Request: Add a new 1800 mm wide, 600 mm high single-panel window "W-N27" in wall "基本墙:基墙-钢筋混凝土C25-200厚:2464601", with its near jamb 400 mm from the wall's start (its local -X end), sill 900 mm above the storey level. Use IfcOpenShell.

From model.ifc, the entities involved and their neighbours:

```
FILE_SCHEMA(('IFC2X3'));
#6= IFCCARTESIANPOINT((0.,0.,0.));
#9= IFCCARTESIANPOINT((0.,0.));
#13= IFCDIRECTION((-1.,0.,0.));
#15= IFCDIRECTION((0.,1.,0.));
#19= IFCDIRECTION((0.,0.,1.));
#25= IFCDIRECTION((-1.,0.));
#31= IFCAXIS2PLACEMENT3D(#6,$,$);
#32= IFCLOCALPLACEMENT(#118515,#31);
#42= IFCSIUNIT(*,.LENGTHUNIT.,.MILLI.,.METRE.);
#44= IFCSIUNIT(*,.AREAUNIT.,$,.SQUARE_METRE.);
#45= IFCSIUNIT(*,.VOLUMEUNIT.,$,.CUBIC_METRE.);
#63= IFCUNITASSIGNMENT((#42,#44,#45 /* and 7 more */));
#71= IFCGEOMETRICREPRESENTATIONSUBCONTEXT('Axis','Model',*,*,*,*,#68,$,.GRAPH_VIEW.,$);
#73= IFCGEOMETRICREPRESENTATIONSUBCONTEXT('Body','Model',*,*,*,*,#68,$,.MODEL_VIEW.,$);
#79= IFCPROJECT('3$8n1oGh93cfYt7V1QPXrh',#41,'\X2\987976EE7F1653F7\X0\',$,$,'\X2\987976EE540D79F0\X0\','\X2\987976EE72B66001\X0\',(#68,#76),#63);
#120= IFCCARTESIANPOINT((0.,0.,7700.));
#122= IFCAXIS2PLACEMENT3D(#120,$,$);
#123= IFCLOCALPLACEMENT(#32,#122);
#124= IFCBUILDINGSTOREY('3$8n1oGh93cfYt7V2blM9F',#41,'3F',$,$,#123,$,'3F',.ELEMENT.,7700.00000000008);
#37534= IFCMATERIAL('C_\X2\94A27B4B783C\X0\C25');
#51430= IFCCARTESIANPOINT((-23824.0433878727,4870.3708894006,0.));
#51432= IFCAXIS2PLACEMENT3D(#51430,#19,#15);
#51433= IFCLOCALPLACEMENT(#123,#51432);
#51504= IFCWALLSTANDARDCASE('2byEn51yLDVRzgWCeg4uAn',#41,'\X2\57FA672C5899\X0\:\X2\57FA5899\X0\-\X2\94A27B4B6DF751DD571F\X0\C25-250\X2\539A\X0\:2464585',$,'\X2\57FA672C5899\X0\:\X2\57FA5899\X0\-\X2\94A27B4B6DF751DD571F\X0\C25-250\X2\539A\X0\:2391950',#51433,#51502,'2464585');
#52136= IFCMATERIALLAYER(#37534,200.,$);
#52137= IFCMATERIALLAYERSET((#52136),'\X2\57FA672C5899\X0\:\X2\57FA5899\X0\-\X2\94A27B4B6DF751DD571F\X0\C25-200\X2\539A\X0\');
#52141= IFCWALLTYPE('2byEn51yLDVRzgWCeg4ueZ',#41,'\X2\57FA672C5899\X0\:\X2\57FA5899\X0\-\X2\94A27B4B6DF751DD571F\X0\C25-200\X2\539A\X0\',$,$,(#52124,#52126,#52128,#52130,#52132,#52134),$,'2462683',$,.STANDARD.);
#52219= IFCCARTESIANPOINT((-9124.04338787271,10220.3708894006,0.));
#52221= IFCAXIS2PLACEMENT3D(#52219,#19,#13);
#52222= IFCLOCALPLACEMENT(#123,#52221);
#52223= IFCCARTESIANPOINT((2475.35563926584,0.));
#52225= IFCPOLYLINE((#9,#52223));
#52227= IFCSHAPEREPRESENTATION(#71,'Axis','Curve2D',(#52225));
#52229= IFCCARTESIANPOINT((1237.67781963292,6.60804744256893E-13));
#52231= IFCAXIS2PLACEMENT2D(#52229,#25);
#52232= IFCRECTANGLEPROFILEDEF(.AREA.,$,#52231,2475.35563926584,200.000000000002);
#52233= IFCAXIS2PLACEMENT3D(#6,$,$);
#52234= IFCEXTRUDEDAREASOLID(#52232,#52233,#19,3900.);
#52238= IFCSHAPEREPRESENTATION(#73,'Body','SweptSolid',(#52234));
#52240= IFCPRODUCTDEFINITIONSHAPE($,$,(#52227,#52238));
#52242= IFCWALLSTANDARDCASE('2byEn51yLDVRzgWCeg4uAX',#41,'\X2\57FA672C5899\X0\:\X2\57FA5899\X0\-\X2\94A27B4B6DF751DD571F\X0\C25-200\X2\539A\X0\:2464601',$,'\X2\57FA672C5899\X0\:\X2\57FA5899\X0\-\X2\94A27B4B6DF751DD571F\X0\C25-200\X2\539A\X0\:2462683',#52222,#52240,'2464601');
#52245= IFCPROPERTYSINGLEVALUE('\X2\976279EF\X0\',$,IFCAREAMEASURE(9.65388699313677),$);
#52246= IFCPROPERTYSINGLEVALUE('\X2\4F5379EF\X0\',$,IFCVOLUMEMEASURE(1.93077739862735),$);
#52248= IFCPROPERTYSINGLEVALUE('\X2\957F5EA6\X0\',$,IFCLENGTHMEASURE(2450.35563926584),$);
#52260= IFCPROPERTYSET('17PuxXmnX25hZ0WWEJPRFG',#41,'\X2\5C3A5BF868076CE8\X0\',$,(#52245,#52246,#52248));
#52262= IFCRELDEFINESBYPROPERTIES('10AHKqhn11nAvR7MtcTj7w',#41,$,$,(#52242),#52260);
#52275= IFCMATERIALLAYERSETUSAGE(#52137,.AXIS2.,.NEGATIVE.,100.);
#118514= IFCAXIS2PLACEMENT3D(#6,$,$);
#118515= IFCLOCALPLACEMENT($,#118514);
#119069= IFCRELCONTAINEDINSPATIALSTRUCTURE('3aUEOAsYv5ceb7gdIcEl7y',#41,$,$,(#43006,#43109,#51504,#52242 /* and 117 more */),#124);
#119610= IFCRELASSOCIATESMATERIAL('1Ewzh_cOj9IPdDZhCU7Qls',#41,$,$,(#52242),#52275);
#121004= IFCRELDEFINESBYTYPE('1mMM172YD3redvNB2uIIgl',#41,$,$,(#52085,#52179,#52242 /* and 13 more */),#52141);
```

```python
import numpy as np
import ifcopenshell
import ifcopenshell.api.feature
import ifcopenshell.api.geometry
import ifcopenshell.api.pset
import ifcopenshell.api.root
import ifcopenshell.api.spatial
import ifcopenshell.api.type
import ifcopenshell.geom
import ifcopenshell.util.element
import ifcopenshell.util.placement
import ifcopenshell.util.representation
import ifcopenshell.util.shape
import ifcopenshell.util.unit

model = ifcopenshell.open("model.ifc")
unit_scale = ifcopenshell.util.unit.calculate_unit_scale(model)
area_scale = ifcopenshell.util.unit.calculate_unit_scale(model, "AREAUNIT")
volume_scale = ifcopenshell.util.unit.calculate_unit_scale(model, "VOLUMEUNIT")
settings = ifcopenshell.geom.settings()


def volume(element):
    """Net volume in cubic metres, openings subtracted."""
    shape = ifcopenshell.geom.create_shape(settings, element)
    return ifcopenshell.util.shape.get_volume(shape.geometry)


wall = model.by_guid("2byEn51yLDVRzgWCeg4uAX")
storey = ifcopenshell.util.element.get_container(wall, ifc_class="IfcBuildingStorey")
context = ifcopenshell.util.representation.get_context(model, "Model", "Body", "MODEL_VIEW")
before = volume(wall)

width, height, from_end, sill = 1.8, 0.6, 0.4, 0.9  # metres

# The wall runs along its own X axis, and the end named is its -X end.
wall_shape = ifcopenshell.geom.create_shape(settings, wall)
x, y, z = ifcopenshell.util.shape.get_vertices(wall_shape.geometry).T
start = x.min() + from_end
face, thickness = float(y.min()), float(y.max() - y.min())
wall_matrix = ifcopenshell.util.placement.get_local_placement(wall.ObjectPlacement)
level = ifcopenshell.util.placement.get_local_placement(storey.ObjectPlacement)[2, 3]


def in_wall(x, y):
    """Placement at x, y metres in the wall's axes, at sill height."""
    matrix = wall_matrix.copy()
    matrix[:, 3] = wall_matrix @ np.array([x / unit_scale, y / unit_scale, 0.0, 1.0])
    matrix[2, 3] = level + sill / unit_scale
    return matrix


# Opening: a box that overshoots both wall faces by 50 mm.
opening = ifcopenshell.api.root.create_entity(model, ifc_class="IfcOpeningElement")
box = ifcopenshell.api.geometry.add_wall_representation(
    model, context=context, length=width, height=height, thickness=thickness + 0.1
)
ifcopenshell.api.geometry.assign_representation(model, product=opening, representation=box)
ifcopenshell.api.geometry.edit_object_placement(model, product=opening, matrix=in_wall(start, face - 0.05), is_si=False)
ifcopenshell.api.feature.add_feature(model, feature=opening, element=wall)

window = ifcopenshell.api.root.create_entity(model, ifc_class="IfcWindow", name="W-N27")
window.OverallWidth, window.OverallHeight = width / unit_scale, height / unit_scale
body = ifcopenshell.api.geometry.add_window_representation(
    model,
    context=context,
    overall_width=window.OverallWidth,
    overall_height=window.OverallHeight,
    partition_type="SINGLE_PANEL",
)
ifcopenshell.api.geometry.assign_representation(model, product=window, representation=body)
ifcopenshell.api.spatial.assign_container(model, products=[window], relating_structure=storey)
fills = ifcopenshell.api.feature.add_filling(model, opening=opening, element=window)
fills.OwnerHistory = window.OwnerHistory  # required in IFC2X3

# IFC2X3 keeps the operation on the window style.
style = ifcopenshell.api.root.create_entity(model, ifc_class="IfcWindowStyle", name="W-N27")
style.OperationType, style.ConstructionType = "SINGLE_PANEL", "NOTDEFINED"
style.ParameterTakesPrecedence = style.Sizeable = False
ifcopenshell.api.type.assign_type(model, related_objects=[window], relating_type=style)

# Centre the window in the wall's thickness.
ifcopenshell.api.geometry.edit_object_placement(model, product=window, matrix=in_wall(start, face), is_si=False)
window_shape = ifcopenshell.geom.create_shape(settings, window)
depth = ifcopenshell.util.shape.get_vertices(window_shape.geometry)[:, 1]
offset = face + thickness / 2 - (depth.min() + depth.max()) / 2
ifcopenshell.api.geometry.edit_object_placement(model, product=window, matrix=in_wall(start, offset), is_si=False)

after = volume(wall)

# Update the wall's stored quantities.
pset = model.by_id(ifcopenshell.util.element.get_pset(wall, "尺寸标注", should_inherit=False)["id"])
ifcopenshell.api.pset.edit_pset(model, pset=pset, properties={
    "面积": model.create_entity("IfcAreaMeasure", after / thickness / area_scale),
    "体积": model.create_entity("IfcVolumeMeasure", after / volume_scale),
})

print(f"wall volume {before:.3f} -> {after:.3f} m3")

model.write("model_rev.ifc")
```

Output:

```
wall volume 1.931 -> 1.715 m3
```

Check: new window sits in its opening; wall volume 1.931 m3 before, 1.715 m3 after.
